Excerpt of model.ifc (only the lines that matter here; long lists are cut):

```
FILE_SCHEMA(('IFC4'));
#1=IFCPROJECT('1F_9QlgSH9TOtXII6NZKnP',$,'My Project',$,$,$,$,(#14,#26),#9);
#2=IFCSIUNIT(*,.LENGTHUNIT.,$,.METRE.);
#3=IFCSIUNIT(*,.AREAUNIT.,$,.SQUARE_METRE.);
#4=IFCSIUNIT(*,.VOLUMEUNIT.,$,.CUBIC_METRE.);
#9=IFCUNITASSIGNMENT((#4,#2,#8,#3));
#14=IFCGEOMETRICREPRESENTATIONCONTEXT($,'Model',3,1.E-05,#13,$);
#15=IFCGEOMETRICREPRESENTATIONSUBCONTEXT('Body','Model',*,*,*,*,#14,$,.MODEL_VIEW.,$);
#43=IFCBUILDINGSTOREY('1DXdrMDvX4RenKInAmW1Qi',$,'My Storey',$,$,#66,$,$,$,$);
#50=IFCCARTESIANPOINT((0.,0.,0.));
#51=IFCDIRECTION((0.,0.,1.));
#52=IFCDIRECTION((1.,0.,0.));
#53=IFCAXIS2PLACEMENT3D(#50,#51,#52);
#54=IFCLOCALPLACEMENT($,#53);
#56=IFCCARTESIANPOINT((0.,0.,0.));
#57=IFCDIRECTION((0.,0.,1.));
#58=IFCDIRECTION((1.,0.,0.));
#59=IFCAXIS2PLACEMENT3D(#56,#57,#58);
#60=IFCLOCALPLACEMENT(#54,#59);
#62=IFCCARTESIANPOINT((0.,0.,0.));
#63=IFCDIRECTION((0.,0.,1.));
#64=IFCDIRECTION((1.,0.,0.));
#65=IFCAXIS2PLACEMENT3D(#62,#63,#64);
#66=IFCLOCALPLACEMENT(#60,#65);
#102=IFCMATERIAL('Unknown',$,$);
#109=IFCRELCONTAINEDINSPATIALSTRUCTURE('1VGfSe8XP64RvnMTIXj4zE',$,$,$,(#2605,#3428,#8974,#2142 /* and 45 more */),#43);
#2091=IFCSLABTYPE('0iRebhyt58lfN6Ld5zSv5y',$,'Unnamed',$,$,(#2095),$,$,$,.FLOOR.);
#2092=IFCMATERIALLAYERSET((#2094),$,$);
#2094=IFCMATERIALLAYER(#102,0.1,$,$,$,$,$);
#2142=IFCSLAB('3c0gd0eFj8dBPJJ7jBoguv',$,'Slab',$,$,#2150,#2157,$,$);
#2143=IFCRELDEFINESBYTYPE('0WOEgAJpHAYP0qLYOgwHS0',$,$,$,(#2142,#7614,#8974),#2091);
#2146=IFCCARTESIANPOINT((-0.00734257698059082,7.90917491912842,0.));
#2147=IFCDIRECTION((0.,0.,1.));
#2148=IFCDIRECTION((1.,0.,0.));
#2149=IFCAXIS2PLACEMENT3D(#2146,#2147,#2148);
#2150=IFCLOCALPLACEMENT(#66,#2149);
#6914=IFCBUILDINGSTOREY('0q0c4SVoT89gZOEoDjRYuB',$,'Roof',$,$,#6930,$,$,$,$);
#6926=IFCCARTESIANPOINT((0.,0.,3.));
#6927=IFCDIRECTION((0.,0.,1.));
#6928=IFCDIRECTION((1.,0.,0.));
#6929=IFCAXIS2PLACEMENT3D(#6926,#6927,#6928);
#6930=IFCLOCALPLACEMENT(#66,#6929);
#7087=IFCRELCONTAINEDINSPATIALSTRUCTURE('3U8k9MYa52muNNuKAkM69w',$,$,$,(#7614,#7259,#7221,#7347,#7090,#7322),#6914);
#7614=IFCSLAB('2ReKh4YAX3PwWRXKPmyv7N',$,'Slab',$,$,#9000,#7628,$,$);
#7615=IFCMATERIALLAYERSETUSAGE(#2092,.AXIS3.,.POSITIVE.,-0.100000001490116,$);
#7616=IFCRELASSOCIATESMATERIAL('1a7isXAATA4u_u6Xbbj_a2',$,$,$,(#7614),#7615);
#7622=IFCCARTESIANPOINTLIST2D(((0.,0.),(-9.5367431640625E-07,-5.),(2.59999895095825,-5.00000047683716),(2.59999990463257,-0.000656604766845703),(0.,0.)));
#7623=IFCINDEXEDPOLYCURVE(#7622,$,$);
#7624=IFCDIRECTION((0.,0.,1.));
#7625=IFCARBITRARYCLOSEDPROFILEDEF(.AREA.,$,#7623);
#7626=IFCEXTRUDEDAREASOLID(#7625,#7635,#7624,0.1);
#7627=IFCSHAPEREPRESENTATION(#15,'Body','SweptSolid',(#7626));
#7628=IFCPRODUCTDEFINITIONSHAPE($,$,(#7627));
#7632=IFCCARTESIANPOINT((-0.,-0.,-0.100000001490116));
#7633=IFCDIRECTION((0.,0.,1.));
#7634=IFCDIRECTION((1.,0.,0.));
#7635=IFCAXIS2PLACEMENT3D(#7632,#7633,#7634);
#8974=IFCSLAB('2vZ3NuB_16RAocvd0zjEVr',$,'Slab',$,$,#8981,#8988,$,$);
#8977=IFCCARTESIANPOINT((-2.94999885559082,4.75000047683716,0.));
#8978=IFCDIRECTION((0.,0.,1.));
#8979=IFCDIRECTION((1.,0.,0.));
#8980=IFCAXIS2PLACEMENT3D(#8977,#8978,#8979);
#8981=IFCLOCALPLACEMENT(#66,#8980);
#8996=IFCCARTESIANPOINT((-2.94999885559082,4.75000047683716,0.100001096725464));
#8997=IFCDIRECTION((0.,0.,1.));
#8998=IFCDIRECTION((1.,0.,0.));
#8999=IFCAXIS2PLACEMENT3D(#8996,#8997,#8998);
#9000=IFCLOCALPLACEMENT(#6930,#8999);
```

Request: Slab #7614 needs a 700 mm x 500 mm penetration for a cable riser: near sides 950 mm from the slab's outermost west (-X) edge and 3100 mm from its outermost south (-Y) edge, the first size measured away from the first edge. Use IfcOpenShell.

```python
import numpy as np
import ifcopenshell
import ifcopenshell.api.feature
import ifcopenshell.api.geometry
import ifcopenshell.api.root
import ifcopenshell.geom
import ifcopenshell.util.placement
import ifcopenshell.util.representation
import ifcopenshell.util.shape
import ifcopenshell.util.unit

model = ifcopenshell.open("model.ifc")
unit_scale = ifcopenshell.util.unit.calculate_unit_scale(model)
settings = ifcopenshell.geom.settings()


def volume(element):
    """Net volume in cubic metres, openings subtracted."""
    shape = ifcopenshell.geom.create_shape(settings, element)
    return ifcopenshell.util.shape.get_volume(shape.geometry)


slab = model.by_guid("2ReKh4YAX3PwWRXKPmyv7N")
before = volume(slab)

# Extent in the slab's own axes, in metres. The edges named are its -X and -Y sides.
slab_shape = ifcopenshell.geom.create_shape(settings, slab)
vertices = ifcopenshell.util.shape.get_vertices(slab_shape.geometry)
x_min, y_min, bottom = vertices.min(axis=0)
top = vertices[:, 2].max()

opening = ifcopenshell.api.root.create_entity(model, ifc_class="IfcOpeningElement", name="Cable riser opening", predefined_type="OPENING")
context = ifcopenshell.util.representation.get_context(model, "Model", "Body", "MODEL_VIEW")
width, depth = 0.7, 0.5
outline = [(0.0, 0.0), (width, 0.0), (width, depth), (0.0, depth), (0.0, 0.0)]
# Overshoot both faces by 50 mm so the cut is clean.
shape = ifcopenshell.api.geometry.add_slab_representation(
    model, context=context, depth=top - bottom + 0.1, polyline=outline
)
ifcopenshell.api.geometry.assign_representation(model, product=opening, representation=shape)

matrix = ifcopenshell.util.placement.get_local_placement(slab.ObjectPlacement)
matrix[:, 3] = matrix @ np.append(np.array([x_min + 0.95, y_min + 3.1, bottom - 0.05]) / unit_scale, 1.0)
ifcopenshell.api.geometry.edit_object_placement(model, product=opening, matrix=matrix, is_si=False)
ifcopenshell.api.feature.add_feature(model, feature=opening, element=slab)

after = volume(slab)

print(f"slab volume {before:.3f} -> {after:.3f} m3")

model.write("model_rev.ifc")
```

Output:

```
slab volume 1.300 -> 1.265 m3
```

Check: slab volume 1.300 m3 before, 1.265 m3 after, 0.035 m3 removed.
